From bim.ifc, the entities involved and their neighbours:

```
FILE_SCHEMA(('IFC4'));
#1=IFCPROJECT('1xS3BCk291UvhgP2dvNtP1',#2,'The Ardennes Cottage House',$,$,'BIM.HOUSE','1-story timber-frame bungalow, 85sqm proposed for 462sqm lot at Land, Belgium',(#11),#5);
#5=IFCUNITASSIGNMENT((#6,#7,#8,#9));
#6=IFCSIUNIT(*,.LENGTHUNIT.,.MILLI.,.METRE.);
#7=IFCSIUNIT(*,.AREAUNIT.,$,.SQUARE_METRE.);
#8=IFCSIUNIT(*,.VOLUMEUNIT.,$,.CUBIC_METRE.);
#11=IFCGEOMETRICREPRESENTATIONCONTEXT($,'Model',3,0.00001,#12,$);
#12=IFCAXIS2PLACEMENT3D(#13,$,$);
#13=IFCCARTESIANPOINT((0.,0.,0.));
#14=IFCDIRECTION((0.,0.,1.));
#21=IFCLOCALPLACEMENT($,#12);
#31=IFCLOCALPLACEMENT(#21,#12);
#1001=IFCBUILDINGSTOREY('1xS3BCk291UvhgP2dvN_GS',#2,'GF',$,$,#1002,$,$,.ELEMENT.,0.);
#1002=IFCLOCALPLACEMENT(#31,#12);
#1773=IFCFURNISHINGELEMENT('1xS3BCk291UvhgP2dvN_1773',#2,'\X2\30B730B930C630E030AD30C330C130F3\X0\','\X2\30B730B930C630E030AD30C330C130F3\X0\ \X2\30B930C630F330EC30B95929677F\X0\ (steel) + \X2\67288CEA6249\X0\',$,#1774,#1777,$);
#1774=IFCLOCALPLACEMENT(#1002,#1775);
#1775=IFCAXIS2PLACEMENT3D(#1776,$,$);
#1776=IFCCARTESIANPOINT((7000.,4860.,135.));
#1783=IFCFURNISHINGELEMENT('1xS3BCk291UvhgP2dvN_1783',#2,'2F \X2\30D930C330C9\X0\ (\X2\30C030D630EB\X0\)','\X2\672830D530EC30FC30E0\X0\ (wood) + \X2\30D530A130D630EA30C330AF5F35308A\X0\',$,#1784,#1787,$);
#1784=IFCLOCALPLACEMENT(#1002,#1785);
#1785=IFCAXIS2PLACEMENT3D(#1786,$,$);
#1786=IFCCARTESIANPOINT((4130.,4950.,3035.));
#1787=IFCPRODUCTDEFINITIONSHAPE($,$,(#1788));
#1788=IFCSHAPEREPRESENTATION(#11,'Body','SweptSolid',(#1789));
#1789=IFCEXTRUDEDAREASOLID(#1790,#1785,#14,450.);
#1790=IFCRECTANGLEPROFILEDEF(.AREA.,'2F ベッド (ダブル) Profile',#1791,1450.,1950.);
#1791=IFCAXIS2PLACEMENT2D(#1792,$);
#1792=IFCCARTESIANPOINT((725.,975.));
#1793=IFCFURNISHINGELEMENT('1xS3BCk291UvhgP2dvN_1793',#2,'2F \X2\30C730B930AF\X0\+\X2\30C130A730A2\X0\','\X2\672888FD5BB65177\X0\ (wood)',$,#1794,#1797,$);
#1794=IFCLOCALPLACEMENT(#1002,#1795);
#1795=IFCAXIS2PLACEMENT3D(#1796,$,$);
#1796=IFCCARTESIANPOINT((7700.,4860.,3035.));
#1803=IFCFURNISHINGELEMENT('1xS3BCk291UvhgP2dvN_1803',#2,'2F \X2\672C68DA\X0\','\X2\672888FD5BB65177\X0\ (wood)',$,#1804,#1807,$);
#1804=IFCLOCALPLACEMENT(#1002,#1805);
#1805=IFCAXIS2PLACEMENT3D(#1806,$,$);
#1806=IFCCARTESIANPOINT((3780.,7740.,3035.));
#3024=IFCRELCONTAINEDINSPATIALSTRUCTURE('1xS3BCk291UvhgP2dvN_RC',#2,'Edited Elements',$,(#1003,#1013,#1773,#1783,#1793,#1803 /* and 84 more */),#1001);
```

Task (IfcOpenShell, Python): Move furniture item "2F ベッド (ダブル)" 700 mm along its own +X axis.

```python
import ifcopenshell
import ifcopenshell.api.geometry
import ifcopenshell.util.placement
import ifcopenshell.util.unit

model = ifcopenshell.open("bim.ifc")
unit_scale = ifcopenshell.util.unit.calculate_unit_scale(model)

item = model.by_id(1783)
matrix = ifcopenshell.util.placement.get_local_placement(item.ObjectPlacement)
matrix[:3, 3] += matrix[:3, 0] * 0.7 / unit_scale
ifcopenshell.api.geometry.edit_object_placement(model, product=item, matrix=matrix, is_si=False)

print(ifcopenshell.util.placement.get_local_placement(item.ObjectPlacement).round(3) + 0.0)

model.write("bim-out.ifc")
```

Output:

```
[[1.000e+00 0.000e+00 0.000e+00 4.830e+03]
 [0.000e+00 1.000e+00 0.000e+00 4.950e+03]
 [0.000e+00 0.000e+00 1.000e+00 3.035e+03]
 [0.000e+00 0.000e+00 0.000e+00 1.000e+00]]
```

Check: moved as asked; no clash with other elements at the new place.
